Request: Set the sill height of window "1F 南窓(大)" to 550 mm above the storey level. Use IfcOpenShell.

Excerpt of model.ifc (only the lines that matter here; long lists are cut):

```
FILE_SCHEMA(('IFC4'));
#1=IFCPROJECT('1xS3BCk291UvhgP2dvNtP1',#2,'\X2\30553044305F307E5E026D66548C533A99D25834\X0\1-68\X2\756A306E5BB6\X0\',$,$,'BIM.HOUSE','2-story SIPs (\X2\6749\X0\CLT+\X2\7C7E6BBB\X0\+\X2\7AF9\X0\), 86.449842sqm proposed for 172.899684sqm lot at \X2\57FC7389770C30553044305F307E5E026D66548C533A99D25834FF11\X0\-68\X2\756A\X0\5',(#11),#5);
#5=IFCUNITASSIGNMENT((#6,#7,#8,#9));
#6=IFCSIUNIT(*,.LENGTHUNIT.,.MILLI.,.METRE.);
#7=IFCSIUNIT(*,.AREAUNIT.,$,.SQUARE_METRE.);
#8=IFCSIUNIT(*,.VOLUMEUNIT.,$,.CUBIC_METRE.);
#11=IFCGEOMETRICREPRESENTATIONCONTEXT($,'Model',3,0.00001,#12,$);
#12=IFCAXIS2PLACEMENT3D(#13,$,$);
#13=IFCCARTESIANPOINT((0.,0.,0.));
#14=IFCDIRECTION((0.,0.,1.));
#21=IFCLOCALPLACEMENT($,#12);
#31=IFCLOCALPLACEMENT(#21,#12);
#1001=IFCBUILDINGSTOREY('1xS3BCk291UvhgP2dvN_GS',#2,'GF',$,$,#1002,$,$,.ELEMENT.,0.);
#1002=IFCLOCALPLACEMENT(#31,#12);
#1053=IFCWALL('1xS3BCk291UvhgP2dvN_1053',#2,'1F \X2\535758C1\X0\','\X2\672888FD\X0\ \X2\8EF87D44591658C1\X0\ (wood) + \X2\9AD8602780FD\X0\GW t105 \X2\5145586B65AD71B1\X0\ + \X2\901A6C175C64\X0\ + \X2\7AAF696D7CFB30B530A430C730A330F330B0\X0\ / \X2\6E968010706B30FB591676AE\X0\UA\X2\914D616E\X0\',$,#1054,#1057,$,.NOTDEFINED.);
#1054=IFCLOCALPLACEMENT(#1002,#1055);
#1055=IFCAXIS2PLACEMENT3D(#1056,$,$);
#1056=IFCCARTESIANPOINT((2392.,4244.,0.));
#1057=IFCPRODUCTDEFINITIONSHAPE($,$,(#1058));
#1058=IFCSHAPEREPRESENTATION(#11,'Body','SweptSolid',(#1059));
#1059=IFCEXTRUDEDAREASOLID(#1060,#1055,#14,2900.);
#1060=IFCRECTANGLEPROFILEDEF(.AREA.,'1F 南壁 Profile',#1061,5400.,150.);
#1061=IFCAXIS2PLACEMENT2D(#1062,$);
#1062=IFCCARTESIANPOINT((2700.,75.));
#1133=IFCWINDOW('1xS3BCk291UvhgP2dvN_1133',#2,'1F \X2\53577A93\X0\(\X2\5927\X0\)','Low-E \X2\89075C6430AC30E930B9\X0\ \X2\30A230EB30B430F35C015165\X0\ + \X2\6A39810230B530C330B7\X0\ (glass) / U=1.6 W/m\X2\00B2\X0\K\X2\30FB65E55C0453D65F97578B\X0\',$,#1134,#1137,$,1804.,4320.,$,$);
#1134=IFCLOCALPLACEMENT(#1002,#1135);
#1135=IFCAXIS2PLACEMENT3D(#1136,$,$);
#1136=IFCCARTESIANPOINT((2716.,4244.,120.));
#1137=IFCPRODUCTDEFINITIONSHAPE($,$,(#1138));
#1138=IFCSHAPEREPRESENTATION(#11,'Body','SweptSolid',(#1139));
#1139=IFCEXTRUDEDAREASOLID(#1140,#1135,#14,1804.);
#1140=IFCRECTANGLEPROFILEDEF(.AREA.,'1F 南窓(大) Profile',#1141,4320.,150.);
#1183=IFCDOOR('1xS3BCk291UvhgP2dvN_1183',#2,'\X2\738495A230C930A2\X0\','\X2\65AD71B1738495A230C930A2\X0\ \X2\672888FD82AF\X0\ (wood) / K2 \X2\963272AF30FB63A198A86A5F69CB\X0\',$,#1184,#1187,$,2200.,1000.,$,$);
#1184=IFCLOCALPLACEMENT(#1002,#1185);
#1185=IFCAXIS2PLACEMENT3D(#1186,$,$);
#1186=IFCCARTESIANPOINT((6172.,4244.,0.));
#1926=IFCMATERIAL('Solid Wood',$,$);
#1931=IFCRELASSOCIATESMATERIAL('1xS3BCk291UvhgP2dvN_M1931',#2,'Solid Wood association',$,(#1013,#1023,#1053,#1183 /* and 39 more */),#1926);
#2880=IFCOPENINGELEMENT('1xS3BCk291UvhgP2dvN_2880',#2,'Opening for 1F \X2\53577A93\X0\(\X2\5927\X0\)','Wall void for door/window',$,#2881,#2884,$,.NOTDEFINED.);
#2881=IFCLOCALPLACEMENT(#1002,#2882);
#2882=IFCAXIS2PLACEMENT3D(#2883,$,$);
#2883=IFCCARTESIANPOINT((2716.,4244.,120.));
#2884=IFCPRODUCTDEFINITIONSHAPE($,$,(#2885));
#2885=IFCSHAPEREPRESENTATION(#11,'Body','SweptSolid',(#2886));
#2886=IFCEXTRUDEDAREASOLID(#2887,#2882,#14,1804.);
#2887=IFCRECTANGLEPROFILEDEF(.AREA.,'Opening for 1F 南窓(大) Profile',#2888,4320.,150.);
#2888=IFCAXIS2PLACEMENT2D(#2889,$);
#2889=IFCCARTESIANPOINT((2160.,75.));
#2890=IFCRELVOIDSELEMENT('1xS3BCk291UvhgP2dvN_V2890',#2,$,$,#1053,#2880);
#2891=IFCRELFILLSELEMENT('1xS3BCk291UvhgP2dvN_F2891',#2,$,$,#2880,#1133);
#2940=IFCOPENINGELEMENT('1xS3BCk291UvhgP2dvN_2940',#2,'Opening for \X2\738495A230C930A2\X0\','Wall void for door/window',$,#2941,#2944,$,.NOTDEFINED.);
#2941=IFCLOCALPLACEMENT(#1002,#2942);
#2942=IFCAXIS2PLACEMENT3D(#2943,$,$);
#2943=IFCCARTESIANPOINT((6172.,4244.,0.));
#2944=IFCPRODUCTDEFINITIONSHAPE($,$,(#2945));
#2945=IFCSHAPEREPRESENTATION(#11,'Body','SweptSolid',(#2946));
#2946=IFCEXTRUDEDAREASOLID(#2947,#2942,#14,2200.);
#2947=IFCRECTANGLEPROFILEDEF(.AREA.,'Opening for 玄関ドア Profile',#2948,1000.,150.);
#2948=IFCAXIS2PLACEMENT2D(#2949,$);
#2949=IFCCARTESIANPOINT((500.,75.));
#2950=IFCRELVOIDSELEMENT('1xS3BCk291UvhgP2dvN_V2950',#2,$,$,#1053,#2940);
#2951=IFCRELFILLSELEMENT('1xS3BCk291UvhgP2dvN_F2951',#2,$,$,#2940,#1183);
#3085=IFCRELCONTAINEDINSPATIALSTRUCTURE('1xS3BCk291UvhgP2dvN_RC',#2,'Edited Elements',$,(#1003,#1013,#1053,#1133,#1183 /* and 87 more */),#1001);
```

```python
import numpy as np
import ifcopenshell
import ifcopenshell.api.geometry
import ifcopenshell.geom
import ifcopenshell.util.element
import ifcopenshell.util.placement
import ifcopenshell.util.shape
import ifcopenshell.util.unit

model = ifcopenshell.open("model.ifc")
unit_scale = ifcopenshell.util.unit.calculate_unit_scale(model)

window = model.by_guid("1xS3BCk291UvhgP2dvN_1133")
opening = window.FillsVoids[0].RelatingOpeningElement
storey = ifcopenshell.util.element.get_container(window, ifc_class="IfcBuildingStorey")
level = ifcopenshell.util.placement.get_local_placement(storey.ObjectPlacement)[2, 3]

# The opening's origin need not be at the sill, so measure its lowest point.
shape = ifcopenshell.geom.create_shape(ifcopenshell.geom.settings(), opening)
bottom = ifcopenshell.util.shape.get_shape_bottom_elevation(shape, shape.geometry) / unit_scale
dz = level + 550.0 - bottom

shift = np.array([0.0, 0.0, dz])
# The window is not placed relative to its opening, so move both.
for product in (opening, window):
    matrix = ifcopenshell.util.placement.get_local_placement(product.ObjectPlacement)
    matrix[:3, 3] += shift
    ifcopenshell.api.geometry.edit_object_placement(model, product=product, matrix=matrix, is_si=False)

print(f"moved by {dz * unit_scale:+.3f} m")

model.write("model_rev.ifc")
```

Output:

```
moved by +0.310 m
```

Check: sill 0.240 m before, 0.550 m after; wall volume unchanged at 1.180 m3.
